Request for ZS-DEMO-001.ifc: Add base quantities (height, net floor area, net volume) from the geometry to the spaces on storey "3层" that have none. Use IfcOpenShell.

First a look at what the model holds.

```python
import ifcopenshell
import ifcopenshell.util.element
import ifcopenshell.util.unit

model = ifcopenshell.open("ZS-DEMO-001.ifc")
print(model.schema)
for unit_type in ("LENGTHUNIT", "AREAUNIT", "VOLUMEUNIT"):
    print(unit_type, ifcopenshell.util.unit.calculate_unit_scale(model, unit_type))
storey = next(s for s in model.by_type("IfcBuildingStorey") if s.Name == "3层")
spaces = [e for e in ifcopenshell.util.element.get_decomposition(storey) if e.is_a("IfcSpace")]
for e in sorted(spaces, key=lambda e: e.id()):
    print(e.id(), e.is_a(), e.Name, list(ifcopenshell.util.element.get_psets(e, qtos_only=True)), sep=" | ")
```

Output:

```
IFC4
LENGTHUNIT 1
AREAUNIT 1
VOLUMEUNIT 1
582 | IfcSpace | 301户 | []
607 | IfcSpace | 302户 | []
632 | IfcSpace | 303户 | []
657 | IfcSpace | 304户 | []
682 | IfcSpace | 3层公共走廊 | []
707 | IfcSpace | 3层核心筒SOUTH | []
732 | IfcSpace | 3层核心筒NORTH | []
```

```python
import ifcopenshell
import ifcopenshell.api.pset
import ifcopenshell.geom
import ifcopenshell.util.element
import ifcopenshell.util.shape
import ifcopenshell.util.unit

model = ifcopenshell.open("ZS-DEMO-001.ifc")
unit_scale = ifcopenshell.util.unit.calculate_unit_scale(model)
area_scale = ifcopenshell.util.unit.calculate_unit_scale(model, "AREAUNIT")
volume_scale = ifcopenshell.util.unit.calculate_unit_scale(model, "VOLUMEUNIT")
settings = ifcopenshell.geom.settings()

storey = next(s for s in model.by_type("IfcBuildingStorey") if s.Name == "3层")
spaces = [e for e in ifcopenshell.util.element.get_decomposition(storey) if e.is_a("IfcSpace")]

for e in sorted(spaces, key=lambda e: e.id()):
    if ifcopenshell.util.element.get_psets(e, qtos_only=True, should_inherit=False):
        continue
    # Geometry comes back in metres, in the element's own axes.
    shape = ifcopenshell.geom.create_shape(settings, e)
    values = {
        "Height": ifcopenshell.util.shape.get_z(shape.geometry) / unit_scale,
        "NetFloorArea": ifcopenshell.util.shape.get_footprint_area(shape.geometry) / area_scale,
        "NetVolume": ifcopenshell.util.shape.get_volume(shape.geometry) / volume_scale,
    }
    qto = ifcopenshell.api.pset.add_qto(model, product=e, name="Qto_SpaceBaseQuantities")
    ifcopenshell.api.pset.edit_qto(model, qto=qto, properties=values)
    print(e.id(), {k: round(v, 3) for k, v in values.items()})

model.write("ZS-DEMO-001-out.ifc")
```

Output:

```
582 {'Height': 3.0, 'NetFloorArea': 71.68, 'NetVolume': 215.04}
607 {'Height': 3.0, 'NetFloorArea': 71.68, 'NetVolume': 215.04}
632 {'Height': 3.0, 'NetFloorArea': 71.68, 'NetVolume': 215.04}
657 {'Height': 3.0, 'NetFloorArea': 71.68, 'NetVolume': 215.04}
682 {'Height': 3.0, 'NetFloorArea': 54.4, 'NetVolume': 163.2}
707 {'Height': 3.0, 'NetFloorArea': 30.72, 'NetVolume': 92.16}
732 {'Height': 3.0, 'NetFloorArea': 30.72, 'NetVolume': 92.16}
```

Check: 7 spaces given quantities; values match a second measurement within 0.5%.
